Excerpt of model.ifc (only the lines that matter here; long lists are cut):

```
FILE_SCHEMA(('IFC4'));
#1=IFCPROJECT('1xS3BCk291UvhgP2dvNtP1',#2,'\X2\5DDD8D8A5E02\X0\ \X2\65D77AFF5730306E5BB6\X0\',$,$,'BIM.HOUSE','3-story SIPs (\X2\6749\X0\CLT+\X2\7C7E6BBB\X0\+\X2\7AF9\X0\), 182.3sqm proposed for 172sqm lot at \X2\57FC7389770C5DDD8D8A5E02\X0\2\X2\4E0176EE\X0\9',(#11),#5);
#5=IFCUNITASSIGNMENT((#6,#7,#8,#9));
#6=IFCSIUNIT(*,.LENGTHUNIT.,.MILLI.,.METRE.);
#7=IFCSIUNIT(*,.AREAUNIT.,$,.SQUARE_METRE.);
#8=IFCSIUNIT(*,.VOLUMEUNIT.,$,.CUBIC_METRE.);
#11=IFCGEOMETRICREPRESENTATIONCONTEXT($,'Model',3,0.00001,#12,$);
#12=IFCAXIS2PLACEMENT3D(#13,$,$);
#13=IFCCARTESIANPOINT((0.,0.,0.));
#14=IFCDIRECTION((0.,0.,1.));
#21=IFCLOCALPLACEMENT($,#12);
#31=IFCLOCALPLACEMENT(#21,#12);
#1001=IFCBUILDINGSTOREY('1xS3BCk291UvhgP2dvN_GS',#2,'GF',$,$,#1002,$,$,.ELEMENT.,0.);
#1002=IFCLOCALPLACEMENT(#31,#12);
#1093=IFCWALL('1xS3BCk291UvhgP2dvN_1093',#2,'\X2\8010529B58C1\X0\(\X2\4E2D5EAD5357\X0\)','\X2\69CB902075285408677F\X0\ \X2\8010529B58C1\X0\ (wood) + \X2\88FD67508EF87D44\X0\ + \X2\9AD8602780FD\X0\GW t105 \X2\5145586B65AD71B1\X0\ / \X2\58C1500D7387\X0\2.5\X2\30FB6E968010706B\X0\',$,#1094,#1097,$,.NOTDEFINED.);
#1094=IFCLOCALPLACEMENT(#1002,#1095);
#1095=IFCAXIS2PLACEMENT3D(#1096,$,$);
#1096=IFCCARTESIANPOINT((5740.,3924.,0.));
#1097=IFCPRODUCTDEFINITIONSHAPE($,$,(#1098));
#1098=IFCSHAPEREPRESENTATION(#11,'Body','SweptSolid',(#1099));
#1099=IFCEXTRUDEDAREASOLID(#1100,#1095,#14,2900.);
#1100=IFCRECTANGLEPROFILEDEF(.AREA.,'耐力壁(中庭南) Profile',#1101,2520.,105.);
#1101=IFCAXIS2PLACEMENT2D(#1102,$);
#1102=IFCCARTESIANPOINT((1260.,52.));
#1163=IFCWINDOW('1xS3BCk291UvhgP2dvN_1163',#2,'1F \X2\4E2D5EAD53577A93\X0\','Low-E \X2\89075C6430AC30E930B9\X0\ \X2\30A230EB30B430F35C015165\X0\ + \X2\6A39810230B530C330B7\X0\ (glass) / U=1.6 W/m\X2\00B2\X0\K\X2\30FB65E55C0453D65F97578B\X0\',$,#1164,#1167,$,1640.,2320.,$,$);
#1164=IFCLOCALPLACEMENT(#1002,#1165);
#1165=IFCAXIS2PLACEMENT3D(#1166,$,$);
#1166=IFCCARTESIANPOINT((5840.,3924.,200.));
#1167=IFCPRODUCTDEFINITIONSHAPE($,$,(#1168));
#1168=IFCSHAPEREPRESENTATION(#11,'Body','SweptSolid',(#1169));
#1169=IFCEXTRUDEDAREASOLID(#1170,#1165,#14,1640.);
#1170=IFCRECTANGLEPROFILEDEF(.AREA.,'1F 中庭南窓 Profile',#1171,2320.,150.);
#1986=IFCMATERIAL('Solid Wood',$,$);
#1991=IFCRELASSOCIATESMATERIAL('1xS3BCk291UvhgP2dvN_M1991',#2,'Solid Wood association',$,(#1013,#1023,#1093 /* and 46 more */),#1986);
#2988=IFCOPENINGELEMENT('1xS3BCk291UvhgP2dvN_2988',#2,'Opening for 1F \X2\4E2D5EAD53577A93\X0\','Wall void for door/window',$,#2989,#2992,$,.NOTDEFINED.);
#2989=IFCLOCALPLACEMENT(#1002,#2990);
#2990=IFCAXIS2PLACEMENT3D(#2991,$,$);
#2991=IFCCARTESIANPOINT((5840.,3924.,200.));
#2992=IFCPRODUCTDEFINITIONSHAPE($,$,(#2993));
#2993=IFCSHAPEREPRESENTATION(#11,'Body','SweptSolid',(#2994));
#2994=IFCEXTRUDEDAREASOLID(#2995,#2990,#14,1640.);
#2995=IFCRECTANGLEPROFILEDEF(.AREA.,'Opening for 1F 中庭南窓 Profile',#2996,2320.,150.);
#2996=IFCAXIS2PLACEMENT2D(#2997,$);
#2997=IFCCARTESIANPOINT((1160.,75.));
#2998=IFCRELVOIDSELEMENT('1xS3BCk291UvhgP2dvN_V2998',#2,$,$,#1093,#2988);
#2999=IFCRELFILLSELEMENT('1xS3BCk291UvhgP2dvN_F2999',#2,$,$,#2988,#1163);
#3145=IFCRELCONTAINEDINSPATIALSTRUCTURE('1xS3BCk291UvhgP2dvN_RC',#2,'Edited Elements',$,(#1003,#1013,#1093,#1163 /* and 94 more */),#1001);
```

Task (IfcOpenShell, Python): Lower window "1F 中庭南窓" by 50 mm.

```python
import numpy as np
import ifcopenshell
import ifcopenshell.api.geometry
import ifcopenshell.util.placement
import ifcopenshell.util.unit

model = ifcopenshell.open("model.ifc")
unit_scale = ifcopenshell.util.unit.calculate_unit_scale(model)

window = model.by_guid("1xS3BCk291UvhgP2dvN_1163")
opening = window.FillsVoids[0].RelatingOpeningElement
dz = -0.05 / unit_scale

shift = np.array([0.0, 0.0, dz])
# The window is not placed relative to its opening, so move both.
for product in (opening, window):
    matrix = ifcopenshell.util.placement.get_local_placement(product.ObjectPlacement)
    matrix[:3, 3] += shift
    ifcopenshell.api.geometry.edit_object_placement(model, product=product, matrix=matrix, is_si=False)

print(f"moved by {dz * unit_scale:+.3f} m")

model.write("model_edited.ifc")
```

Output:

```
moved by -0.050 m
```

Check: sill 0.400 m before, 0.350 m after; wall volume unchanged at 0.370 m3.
